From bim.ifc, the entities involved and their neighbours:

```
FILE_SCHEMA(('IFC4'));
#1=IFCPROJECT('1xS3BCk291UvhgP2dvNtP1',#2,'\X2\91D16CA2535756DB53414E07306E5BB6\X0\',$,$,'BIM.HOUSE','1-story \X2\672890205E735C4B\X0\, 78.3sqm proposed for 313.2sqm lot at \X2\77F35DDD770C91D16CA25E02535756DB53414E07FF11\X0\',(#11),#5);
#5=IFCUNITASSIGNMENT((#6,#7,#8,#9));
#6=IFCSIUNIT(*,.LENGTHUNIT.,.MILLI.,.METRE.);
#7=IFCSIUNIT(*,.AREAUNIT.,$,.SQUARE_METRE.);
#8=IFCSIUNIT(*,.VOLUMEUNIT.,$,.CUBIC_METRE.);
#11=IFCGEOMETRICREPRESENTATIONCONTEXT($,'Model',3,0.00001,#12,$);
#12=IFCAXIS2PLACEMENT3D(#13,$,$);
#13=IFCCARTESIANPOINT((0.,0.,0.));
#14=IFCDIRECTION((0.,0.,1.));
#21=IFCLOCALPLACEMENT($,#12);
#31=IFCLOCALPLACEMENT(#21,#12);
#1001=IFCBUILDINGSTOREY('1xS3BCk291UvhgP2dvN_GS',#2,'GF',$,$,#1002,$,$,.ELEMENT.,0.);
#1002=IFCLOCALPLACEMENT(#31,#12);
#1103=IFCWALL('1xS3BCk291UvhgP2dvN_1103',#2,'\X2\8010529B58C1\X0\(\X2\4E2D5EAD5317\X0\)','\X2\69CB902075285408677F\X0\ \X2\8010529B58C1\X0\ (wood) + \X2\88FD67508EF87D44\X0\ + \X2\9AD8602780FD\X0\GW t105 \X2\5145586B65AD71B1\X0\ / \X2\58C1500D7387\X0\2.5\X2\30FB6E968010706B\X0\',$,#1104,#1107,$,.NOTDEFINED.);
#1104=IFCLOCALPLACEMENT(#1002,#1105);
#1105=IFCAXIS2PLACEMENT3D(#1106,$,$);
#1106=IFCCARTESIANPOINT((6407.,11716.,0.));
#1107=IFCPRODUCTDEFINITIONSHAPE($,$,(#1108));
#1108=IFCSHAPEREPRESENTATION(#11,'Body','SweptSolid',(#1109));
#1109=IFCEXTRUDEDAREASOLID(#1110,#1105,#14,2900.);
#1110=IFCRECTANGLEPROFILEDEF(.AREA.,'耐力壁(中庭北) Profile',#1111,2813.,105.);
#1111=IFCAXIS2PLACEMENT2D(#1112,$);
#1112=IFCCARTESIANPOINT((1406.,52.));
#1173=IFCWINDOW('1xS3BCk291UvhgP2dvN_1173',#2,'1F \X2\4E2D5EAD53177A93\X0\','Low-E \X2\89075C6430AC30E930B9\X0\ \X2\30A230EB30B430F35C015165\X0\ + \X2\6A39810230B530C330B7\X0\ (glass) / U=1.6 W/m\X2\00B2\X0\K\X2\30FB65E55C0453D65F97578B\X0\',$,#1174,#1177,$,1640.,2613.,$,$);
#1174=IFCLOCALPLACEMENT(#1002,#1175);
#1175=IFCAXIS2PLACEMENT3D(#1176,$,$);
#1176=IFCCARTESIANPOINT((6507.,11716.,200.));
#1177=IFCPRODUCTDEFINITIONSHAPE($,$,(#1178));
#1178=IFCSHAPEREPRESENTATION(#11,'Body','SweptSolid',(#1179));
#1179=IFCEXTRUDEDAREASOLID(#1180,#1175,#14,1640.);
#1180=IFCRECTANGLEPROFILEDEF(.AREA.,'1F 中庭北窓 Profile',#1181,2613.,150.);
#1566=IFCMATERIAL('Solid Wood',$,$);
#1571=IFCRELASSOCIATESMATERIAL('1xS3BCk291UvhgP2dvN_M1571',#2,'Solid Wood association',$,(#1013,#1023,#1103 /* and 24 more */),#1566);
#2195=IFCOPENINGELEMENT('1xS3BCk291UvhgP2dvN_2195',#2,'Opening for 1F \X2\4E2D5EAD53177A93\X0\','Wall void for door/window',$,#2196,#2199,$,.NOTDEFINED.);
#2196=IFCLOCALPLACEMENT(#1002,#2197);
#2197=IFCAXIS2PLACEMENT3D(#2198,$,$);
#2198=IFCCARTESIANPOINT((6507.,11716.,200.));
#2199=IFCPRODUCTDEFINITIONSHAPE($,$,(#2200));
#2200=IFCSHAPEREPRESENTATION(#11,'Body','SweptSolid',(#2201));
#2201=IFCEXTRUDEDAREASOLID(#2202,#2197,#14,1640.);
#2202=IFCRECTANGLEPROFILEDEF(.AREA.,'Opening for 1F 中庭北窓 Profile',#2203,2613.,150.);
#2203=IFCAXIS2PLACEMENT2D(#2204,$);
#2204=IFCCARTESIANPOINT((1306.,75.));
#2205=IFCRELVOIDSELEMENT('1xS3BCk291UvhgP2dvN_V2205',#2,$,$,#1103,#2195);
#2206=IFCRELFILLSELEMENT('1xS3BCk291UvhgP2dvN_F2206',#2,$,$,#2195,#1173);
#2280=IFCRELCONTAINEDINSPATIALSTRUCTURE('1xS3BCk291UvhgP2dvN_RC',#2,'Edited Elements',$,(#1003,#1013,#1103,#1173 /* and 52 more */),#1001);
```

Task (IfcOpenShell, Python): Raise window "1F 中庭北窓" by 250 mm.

```python
import numpy as np
import ifcopenshell
import ifcopenshell.api.geometry
import ifcopenshell.util.placement
import ifcopenshell.util.unit

model = ifcopenshell.open("bim.ifc")
unit_scale = ifcopenshell.util.unit.calculate_unit_scale(model)

window = model.by_guid("1xS3BCk291UvhgP2dvN_1173")
opening = window.FillsVoids[0].RelatingOpeningElement
dz = 0.25 / unit_scale

shift = np.array([0.0, 0.0, dz])
# The window is not placed relative to its opening, so move both.
for product in (opening, window):
    matrix = ifcopenshell.util.placement.get_local_placement(product.ObjectPlacement)
    matrix[:3, 3] += shift
    ifcopenshell.api.geometry.edit_object_placement(model, product=product, matrix=matrix, is_si=False)

print(f"moved by {dz * unit_scale:+.3f} m")

model.write("bim_rev.ifc")
```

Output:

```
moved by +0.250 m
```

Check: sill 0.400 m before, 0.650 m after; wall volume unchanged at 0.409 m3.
